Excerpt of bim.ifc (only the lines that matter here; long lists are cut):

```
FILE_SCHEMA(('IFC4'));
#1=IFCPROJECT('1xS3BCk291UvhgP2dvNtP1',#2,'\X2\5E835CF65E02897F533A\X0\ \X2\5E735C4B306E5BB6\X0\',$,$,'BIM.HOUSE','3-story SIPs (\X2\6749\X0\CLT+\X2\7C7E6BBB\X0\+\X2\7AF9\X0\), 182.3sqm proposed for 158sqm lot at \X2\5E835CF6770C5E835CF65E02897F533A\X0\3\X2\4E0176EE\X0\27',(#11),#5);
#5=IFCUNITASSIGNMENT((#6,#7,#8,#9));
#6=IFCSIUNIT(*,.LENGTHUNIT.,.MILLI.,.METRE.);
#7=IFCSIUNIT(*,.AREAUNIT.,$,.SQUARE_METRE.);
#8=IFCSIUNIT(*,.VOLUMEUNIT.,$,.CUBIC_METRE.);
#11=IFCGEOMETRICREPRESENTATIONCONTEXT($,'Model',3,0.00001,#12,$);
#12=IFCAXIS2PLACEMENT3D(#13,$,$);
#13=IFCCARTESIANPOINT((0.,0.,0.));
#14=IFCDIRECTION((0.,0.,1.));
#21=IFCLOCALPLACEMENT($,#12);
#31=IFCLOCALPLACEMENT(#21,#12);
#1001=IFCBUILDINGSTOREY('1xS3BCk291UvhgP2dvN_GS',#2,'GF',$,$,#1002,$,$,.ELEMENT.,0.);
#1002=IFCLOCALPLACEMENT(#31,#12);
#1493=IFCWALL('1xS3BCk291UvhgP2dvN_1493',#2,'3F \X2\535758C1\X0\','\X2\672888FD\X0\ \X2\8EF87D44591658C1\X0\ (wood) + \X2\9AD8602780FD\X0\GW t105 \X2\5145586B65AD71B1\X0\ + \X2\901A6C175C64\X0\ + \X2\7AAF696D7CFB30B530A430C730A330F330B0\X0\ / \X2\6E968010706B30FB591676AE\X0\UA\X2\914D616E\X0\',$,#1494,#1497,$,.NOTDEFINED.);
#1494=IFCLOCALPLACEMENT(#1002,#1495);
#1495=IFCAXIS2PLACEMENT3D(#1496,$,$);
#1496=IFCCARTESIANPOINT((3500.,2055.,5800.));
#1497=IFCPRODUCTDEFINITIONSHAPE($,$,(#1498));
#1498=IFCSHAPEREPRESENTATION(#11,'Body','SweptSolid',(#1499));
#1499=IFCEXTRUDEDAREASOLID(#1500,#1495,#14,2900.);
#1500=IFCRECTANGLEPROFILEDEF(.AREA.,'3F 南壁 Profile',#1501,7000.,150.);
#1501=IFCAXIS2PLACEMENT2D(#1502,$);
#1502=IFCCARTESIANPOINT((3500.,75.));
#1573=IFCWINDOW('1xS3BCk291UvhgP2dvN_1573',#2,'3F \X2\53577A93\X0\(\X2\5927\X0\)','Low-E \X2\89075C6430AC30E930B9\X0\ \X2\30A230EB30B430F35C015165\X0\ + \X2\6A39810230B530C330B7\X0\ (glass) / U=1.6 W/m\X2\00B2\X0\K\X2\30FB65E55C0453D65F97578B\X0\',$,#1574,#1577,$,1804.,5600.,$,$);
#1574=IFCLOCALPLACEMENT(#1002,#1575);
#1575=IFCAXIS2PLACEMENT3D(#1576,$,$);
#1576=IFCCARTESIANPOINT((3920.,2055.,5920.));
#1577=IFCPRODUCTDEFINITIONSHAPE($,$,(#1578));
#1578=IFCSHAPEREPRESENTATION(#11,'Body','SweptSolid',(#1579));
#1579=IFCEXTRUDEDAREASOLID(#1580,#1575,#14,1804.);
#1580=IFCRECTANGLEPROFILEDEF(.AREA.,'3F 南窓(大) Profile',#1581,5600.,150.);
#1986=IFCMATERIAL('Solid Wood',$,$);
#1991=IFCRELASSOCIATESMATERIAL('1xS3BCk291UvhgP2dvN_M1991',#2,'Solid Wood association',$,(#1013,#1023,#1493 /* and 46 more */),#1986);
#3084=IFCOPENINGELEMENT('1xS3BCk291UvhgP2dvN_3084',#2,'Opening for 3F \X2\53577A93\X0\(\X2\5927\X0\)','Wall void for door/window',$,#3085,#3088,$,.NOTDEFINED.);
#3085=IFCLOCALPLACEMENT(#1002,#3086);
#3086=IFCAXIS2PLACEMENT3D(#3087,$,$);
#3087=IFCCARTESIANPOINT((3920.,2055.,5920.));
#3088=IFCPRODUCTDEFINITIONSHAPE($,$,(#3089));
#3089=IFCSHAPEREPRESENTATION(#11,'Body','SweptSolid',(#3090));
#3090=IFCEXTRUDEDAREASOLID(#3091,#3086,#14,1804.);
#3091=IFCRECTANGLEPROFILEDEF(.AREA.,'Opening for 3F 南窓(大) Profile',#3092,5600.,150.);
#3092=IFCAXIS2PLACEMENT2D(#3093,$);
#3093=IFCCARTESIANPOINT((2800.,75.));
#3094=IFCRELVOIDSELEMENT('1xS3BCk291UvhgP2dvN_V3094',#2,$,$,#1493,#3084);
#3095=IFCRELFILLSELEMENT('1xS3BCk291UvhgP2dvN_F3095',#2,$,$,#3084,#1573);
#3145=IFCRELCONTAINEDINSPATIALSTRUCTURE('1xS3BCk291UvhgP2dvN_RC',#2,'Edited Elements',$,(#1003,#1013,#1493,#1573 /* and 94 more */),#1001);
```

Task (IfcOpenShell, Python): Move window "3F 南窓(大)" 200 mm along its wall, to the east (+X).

```python
import ifcopenshell
import ifcopenshell.api.geometry
import ifcopenshell.util.placement
import ifcopenshell.util.unit

model = ifcopenshell.open("bim.ifc")
unit_scale = ifcopenshell.util.unit.calculate_unit_scale(model)

window = model.by_guid("1xS3BCk291UvhgP2dvN_1573")
opening = window.FillsVoids[0].RelatingOpeningElement
wall = opening.VoidsElements[0].RelatingBuildingElement

wall_matrix = ifcopenshell.util.placement.get_local_placement(wall.ObjectPlacement)
shift = wall_matrix[:3, 0] * 0.2 / unit_scale
before = ifcopenshell.util.placement.get_local_placement(window.ObjectPlacement)[:3, 3].copy()

# The window is not placed relative to its opening, so move both.
for product in (opening, window):
    matrix = ifcopenshell.util.placement.get_local_placement(product.ObjectPlacement)
    matrix[:3, 3] += shift
    ifcopenshell.api.geometry.edit_object_placement(model, product=product, matrix=matrix, is_si=False)

after = ifcopenshell.util.placement.get_local_placement(window.ObjectPlacement)[:3, 3]
print("window moved by", (after - before).round(3) + 0.0)

model.write("bim_v2.ifc")
```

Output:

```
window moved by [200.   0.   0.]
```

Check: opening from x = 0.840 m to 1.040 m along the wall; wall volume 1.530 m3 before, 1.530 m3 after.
